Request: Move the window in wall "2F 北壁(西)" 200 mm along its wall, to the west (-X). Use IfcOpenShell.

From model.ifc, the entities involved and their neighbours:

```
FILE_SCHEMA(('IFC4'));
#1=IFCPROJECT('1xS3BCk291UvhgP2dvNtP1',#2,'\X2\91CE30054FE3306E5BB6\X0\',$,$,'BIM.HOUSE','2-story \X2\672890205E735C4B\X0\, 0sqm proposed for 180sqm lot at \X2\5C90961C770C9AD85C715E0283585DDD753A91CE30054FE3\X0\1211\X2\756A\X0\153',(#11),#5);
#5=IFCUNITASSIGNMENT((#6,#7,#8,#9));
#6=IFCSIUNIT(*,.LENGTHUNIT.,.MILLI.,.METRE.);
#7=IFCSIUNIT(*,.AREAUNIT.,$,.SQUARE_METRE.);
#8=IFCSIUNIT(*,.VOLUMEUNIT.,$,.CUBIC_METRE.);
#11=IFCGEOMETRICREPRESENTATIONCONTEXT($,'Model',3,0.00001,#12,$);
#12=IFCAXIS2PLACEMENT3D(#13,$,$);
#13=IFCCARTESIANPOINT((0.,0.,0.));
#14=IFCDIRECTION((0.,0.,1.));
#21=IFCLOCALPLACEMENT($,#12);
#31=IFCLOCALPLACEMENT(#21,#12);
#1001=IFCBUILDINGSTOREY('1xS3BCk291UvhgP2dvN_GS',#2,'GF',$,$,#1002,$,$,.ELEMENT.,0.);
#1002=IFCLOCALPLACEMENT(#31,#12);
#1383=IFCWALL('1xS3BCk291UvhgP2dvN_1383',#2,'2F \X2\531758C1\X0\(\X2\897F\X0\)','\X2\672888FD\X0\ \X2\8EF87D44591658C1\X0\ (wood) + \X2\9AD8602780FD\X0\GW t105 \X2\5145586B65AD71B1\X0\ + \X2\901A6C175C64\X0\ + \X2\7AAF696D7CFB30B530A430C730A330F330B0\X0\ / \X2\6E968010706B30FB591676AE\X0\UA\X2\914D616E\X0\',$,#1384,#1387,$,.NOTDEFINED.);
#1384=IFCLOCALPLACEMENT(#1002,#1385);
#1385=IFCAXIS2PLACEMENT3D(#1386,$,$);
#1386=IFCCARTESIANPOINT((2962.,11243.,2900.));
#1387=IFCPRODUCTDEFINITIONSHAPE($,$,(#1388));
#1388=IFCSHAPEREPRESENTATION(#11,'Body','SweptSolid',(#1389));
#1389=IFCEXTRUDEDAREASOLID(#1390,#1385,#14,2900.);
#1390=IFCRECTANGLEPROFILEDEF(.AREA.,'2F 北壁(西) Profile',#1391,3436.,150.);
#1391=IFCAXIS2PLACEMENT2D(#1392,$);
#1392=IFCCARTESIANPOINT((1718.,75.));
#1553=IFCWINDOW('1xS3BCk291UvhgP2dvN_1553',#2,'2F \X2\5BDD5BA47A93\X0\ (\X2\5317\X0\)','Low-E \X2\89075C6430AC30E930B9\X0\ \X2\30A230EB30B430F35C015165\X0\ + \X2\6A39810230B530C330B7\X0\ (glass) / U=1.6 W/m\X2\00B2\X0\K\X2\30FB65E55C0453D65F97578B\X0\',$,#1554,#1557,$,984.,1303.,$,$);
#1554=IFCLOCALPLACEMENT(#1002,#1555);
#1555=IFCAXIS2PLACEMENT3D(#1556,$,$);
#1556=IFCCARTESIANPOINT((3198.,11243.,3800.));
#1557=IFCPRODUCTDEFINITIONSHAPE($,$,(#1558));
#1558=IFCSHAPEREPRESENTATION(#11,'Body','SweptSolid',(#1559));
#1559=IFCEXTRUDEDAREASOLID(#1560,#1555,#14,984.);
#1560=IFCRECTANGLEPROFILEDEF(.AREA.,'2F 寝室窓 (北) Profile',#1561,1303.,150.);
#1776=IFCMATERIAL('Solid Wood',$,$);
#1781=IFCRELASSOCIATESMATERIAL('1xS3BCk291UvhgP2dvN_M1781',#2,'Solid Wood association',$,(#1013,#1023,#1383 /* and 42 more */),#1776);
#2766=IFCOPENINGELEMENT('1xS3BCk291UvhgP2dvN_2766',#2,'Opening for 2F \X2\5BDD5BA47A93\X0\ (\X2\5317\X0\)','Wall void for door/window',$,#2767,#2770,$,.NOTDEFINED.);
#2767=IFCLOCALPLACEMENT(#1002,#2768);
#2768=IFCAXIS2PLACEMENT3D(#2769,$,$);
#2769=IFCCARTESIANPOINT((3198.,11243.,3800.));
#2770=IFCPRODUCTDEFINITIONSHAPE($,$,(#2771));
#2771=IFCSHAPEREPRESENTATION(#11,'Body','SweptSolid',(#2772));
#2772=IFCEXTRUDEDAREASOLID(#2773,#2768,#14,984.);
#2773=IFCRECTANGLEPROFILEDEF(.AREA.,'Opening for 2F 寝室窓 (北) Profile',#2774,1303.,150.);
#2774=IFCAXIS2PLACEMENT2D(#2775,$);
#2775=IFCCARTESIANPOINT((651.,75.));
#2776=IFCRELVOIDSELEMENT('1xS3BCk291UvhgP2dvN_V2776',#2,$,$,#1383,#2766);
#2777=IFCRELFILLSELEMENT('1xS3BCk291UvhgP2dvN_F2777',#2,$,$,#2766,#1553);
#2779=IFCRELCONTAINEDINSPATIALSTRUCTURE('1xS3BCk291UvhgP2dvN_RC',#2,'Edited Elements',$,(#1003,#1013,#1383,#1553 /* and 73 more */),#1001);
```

```python
import ifcopenshell
import ifcopenshell.api.geometry
import ifcopenshell.util.placement

model = ifcopenshell.open("model.ifc")

window = model.by_id(1553)
opening = window.FillsVoids[0].RelatingOpeningElement
wall = opening.VoidsElements[0].RelatingBuildingElement

wall_matrix = ifcopenshell.util.placement.get_local_placement(wall.ObjectPlacement)
shift = wall_matrix[:3, 0] * -200.0
before = ifcopenshell.util.placement.get_local_placement(window.ObjectPlacement)[:3, 3].copy()

# The window is not placed relative to its opening, so move both.
for product in (opening, window):
    matrix = ifcopenshell.util.placement.get_local_placement(product.ObjectPlacement)
    matrix[:3, 3] += shift
    ifcopenshell.api.geometry.edit_object_placement(model, product=product, matrix=matrix, is_si=False)

after = ifcopenshell.util.placement.get_local_placement(window.ObjectPlacement)[:3, 3]
print("window moved by", (after - before).round(3) + 0.0)

model.write("model_edited.ifc")
```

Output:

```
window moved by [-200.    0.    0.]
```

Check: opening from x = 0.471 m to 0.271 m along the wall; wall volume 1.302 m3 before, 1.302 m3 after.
